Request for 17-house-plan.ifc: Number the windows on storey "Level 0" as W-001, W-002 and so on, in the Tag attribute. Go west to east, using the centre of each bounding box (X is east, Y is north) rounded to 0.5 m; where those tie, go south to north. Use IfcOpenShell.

First a look at what the model holds.

```python
import ifcopenshell
import ifcopenshell.util.element
import ifcopenshell.util.placement

model = ifcopenshell.open("17-house-plan.ifc")
print(model.schema)
storey = next(s for s in model.by_type("IfcBuildingStorey") if s.Name == "Level 0")
windows = [e for e in ifcopenshell.util.element.get_decomposition(storey) if e.is_a("IfcWindow")]
for e in sorted(windows, key=lambda e: e.id()):
    origin = ifcopenshell.util.placement.get_local_placement(e.ObjectPlacement)[:3, 3]
    print(e.id(), e.Tag, e.Name, origin.round(2) + 0.0, sep=" | ")
```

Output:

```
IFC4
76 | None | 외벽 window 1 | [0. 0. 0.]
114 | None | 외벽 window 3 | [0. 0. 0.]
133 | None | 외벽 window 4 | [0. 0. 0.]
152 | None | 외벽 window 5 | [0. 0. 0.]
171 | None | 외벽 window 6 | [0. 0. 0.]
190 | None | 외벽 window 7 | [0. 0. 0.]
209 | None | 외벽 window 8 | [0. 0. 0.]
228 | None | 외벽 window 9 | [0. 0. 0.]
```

```python
import ifcopenshell
import ifcopenshell.geom
import ifcopenshell.util.element
import ifcopenshell.util.shape

model = ifcopenshell.open("17-house-plan.ifc")
settings = ifcopenshell.geom.settings()
settings.set("use-world-coords", True)


def centre(element):
    shape = ifcopenshell.geom.create_shape(settings, element)
    return ifcopenshell.util.shape.get_bbox_centroid(shape.geometry)


storey = next(s for s in model.by_type("IfcBuildingStorey") if s.Name == "Level 0")
windows = [e for e in ifcopenshell.util.element.get_decomposition(storey) if e.is_a("IfcWindow")]

# Insertion points can sit at a corner or the storey origin, so sort by the geometry (in metres).
centres = {e: centre(e) for e in windows}
windows.sort(key=lambda e: (round(centres[e][0] / 0.5), centres[e][1]))

for i, e in enumerate(windows, start=1):
    number = f"W-0{i:02d}"
    e.Tag = number
    print(e.id(), number)

model.write("17-house-plan-out.ifc")
```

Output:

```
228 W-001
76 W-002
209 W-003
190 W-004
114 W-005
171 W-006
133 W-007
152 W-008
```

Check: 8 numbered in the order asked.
